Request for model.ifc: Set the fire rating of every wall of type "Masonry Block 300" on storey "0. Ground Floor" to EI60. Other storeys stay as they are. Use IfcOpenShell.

First a look at what the model holds.

```python
import ifcopenshell
import ifcopenshell.util.element

model = ifcopenshell.open("model.ifc")
print(model.schema)
storey = next(s for s in model.by_type("IfcBuildingStorey") if s.Name == "0. Ground Floor")
walls = [e for e in ifcopenshell.util.element.get_decomposition(storey) if e.is_a("IfcWall")]
seen = {}
for e in walls:
    element_type = ifcopenshell.util.element.get_type(e)
    key = (element_type.Name if element_type != e and element_type else None, ifcopenshell.util.element.get_pset(e, "Pset_WallCommon", "FireRating"))
    seen[key] = seen.get(key, 0) + 1
for (name, value), count in sorted(seen.items(), key=str):
    print(count, "x", name, "|", value)
```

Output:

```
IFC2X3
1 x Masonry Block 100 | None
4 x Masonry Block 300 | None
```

```python
import ifcopenshell
import ifcopenshell.api.pset
import ifcopenshell.util.element

model = ifcopenshell.open("model.ifc")

storey = next(s for s in model.by_type("IfcBuildingStorey") if s.Name == "0. Ground Floor")
walls = [e for e in ifcopenshell.util.element.get_decomposition(storey) if e.is_a("IfcWall")]

count = 0
for e in walls:
    element_type = ifcopenshell.util.element.get_type(e)
    if element_type in (None, e) or element_type.Name != "Masonry Block 300":
        continue
    # add_pset returns the element's existing set when there is one.
    pset = ifcopenshell.api.pset.add_pset(model, product=e, name="Pset_WallCommon")
    ifcopenshell.api.pset.edit_pset(model, pset=pset, properties={"FireRating": "EI60"})
    count += 1

print(count, "walls updated")

model.write("model_rev.ifc")
```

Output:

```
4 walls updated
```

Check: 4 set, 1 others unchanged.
